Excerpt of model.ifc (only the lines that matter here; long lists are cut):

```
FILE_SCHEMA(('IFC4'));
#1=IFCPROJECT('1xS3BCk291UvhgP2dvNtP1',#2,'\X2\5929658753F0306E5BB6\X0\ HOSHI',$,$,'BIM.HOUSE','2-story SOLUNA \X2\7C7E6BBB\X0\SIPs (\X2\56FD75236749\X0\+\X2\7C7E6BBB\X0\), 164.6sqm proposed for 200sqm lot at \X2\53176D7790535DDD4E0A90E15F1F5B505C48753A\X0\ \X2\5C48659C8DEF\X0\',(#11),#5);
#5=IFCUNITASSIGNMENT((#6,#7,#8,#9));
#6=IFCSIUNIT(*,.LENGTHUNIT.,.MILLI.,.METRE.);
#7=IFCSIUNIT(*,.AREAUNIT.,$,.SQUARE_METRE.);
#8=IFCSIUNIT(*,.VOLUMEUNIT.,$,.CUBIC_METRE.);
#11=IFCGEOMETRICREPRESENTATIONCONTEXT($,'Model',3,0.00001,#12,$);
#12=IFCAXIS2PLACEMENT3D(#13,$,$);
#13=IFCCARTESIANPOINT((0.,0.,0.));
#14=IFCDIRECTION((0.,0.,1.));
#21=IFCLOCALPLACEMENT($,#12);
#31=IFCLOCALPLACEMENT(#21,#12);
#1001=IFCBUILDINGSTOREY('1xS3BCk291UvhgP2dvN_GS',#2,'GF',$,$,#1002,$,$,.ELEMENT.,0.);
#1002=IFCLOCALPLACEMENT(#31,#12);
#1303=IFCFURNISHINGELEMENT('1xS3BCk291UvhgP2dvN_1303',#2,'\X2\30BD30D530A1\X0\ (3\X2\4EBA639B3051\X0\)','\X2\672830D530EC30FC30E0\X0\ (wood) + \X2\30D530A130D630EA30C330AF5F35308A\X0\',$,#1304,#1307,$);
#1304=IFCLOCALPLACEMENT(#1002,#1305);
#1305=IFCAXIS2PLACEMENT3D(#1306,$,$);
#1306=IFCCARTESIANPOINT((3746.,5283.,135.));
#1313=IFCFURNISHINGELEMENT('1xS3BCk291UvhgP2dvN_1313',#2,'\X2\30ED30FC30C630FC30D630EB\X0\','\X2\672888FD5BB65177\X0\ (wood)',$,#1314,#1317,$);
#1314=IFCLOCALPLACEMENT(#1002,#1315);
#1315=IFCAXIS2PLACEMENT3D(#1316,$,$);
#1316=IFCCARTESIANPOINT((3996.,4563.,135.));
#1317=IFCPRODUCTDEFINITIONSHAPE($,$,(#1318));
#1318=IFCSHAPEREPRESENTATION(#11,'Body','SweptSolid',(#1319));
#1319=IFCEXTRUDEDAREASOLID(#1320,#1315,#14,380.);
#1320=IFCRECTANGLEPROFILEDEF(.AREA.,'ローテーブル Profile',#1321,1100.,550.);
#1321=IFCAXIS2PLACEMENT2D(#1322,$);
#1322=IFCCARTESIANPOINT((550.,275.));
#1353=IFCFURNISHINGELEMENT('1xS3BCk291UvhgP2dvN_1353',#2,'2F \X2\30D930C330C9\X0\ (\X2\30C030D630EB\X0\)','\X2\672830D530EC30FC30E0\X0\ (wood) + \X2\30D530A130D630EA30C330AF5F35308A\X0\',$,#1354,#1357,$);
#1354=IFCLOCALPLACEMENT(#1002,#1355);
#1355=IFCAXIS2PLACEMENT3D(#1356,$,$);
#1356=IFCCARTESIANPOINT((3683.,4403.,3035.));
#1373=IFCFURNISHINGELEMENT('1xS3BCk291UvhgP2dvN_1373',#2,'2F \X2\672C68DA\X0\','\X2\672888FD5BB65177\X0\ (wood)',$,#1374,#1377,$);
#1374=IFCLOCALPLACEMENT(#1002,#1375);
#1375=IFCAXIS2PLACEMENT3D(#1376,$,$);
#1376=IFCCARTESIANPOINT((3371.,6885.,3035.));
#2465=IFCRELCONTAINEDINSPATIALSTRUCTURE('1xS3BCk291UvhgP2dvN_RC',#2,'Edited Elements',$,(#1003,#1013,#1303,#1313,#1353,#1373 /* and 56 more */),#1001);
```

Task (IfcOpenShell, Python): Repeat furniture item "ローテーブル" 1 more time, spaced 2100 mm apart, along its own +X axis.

```python
import ifcopenshell
import ifcopenshell.api.geometry
import ifcopenshell.api.root
import ifcopenshell.util.element
import ifcopenshell.util.placement

model = ifcopenshell.open("model.ifc")


def reuse_history(source, copy):
    """copy_class also copies each property set's owner history, people and application; keep the originals."""
    for rel in copy.IsDefinedBy:
        if rel.is_a("IfcRelDefinesByProperties") and (history := rel.RelatingPropertyDefinition.OwnerHistory):
            rel.RelatingPropertyDefinition.OwnerHistory = source.OwnerHistory
            ifcopenshell.util.element.remove_deep2(model, history)


source = model.by_guid("1xS3BCk291UvhgP2dvN_1313")
base = ifcopenshell.util.placement.get_local_placement(source.ObjectPlacement)
step = base[:3, 0] * 2100.0

for i in range(1, 2):
    copy = ifcopenshell.api.root.copy_class(model, product=source)
    copy.Representation = ifcopenshell.util.element.copy_deep(
        model, source.Representation, exclude=["IfcGeometricRepresentationContext", "IfcRepresentationMap"]
    )
    reuse_history(source, copy)
    matrix = base.copy()
    matrix[:3, 3] += i * step
    print("added at", matrix[:3, 3].round(3) + 0.0)
    ifcopenshell.api.geometry.edit_object_placement(model, product=copy, matrix=matrix, is_si=False)

model.write("model_edited.ifc")
```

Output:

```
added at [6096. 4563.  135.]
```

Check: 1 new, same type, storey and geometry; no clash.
